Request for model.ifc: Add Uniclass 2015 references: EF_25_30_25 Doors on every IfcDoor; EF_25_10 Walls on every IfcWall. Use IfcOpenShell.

First a look at what the model holds.

```python
import ifcopenshell

model = ifcopenshell.open("model.ifc")
print(model.schema)
print("classifications:", [c.Name for c in model.by_type("IfcClassification")])
for ifc_class in ("IfcDoor", "IfcRoof", "IfcStair", "IfcWall", "IfcWindow"):
    print(ifc_class, len(model.by_type(ifc_class)))
```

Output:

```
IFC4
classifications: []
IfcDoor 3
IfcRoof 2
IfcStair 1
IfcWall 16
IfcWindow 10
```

```python
import ifcopenshell
import ifcopenshell.api.classification

model = ifcopenshell.open("model.ifc")

system = ifcopenshell.api.classification.add_classification(model, classification="Uniclass 2015")

codes = {
    "IfcDoor": ("EF_25_30_25", "Doors"),
    "IfcWall": ("EF_25_10", "Walls"),
}
for ifc_class, (code, name) in codes.items():
    products = model.by_type(ifc_class)
    ifcopenshell.api.classification.add_reference(
        model, products=products, classification=system, identification=code, name=name
    )
    print(code, len(products))

model.write("model_rev.ifc")
```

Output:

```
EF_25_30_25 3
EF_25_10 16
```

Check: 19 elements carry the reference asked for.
